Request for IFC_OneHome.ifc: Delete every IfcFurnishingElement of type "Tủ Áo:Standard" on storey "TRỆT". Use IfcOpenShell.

First a look at what the model holds.

```python
import ifcopenshell
import ifcopenshell.util.element

model = ifcopenshell.open("IFC_OneHome.ifc")
print(model.schema)
storey = next(s for s in model.by_type("IfcBuildingStorey") if s.Name == "TRỆT")
furniture = [e for e in ifcopenshell.util.element.get_decomposition(storey) if e.is_a("IfcFurnishingElement")]
seen = {}
for e in furniture:
    element_type = ifcopenshell.util.element.get_type(e)
    name = element_type.Name if element_type not in (None, e) else None
    seen[name] = seen.get(name, 0) + 1
for name, count in sorted(seen.items(), key=str):
    print(count, "x", name)
```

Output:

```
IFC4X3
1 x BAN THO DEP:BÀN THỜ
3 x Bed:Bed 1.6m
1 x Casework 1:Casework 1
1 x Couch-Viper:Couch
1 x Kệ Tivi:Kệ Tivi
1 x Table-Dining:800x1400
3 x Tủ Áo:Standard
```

```python
import ifcopenshell
import ifcopenshell.api.root
import ifcopenshell.util.element

model = ifcopenshell.open("IFC_OneHome.ifc")

storey = next(s for s in model.by_type("IfcBuildingStorey") if s.Name == "TRỆT")
furniture = [e for e in ifcopenshell.util.element.get_decomposition(storey) if e.is_a("IfcFurnishingElement")]
targets = [e for e in furniture if (t := ifcopenshell.util.element.get_type(e)) not in (None, e) and t.Name == "Tủ Áo:Standard"]

for e in targets:
    ifcopenshell.api.root.remove_product(model, product=e)
print(len(targets), "removed")

model.write("IFC_OneHome_edited.ifc")
```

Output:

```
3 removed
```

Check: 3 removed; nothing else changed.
